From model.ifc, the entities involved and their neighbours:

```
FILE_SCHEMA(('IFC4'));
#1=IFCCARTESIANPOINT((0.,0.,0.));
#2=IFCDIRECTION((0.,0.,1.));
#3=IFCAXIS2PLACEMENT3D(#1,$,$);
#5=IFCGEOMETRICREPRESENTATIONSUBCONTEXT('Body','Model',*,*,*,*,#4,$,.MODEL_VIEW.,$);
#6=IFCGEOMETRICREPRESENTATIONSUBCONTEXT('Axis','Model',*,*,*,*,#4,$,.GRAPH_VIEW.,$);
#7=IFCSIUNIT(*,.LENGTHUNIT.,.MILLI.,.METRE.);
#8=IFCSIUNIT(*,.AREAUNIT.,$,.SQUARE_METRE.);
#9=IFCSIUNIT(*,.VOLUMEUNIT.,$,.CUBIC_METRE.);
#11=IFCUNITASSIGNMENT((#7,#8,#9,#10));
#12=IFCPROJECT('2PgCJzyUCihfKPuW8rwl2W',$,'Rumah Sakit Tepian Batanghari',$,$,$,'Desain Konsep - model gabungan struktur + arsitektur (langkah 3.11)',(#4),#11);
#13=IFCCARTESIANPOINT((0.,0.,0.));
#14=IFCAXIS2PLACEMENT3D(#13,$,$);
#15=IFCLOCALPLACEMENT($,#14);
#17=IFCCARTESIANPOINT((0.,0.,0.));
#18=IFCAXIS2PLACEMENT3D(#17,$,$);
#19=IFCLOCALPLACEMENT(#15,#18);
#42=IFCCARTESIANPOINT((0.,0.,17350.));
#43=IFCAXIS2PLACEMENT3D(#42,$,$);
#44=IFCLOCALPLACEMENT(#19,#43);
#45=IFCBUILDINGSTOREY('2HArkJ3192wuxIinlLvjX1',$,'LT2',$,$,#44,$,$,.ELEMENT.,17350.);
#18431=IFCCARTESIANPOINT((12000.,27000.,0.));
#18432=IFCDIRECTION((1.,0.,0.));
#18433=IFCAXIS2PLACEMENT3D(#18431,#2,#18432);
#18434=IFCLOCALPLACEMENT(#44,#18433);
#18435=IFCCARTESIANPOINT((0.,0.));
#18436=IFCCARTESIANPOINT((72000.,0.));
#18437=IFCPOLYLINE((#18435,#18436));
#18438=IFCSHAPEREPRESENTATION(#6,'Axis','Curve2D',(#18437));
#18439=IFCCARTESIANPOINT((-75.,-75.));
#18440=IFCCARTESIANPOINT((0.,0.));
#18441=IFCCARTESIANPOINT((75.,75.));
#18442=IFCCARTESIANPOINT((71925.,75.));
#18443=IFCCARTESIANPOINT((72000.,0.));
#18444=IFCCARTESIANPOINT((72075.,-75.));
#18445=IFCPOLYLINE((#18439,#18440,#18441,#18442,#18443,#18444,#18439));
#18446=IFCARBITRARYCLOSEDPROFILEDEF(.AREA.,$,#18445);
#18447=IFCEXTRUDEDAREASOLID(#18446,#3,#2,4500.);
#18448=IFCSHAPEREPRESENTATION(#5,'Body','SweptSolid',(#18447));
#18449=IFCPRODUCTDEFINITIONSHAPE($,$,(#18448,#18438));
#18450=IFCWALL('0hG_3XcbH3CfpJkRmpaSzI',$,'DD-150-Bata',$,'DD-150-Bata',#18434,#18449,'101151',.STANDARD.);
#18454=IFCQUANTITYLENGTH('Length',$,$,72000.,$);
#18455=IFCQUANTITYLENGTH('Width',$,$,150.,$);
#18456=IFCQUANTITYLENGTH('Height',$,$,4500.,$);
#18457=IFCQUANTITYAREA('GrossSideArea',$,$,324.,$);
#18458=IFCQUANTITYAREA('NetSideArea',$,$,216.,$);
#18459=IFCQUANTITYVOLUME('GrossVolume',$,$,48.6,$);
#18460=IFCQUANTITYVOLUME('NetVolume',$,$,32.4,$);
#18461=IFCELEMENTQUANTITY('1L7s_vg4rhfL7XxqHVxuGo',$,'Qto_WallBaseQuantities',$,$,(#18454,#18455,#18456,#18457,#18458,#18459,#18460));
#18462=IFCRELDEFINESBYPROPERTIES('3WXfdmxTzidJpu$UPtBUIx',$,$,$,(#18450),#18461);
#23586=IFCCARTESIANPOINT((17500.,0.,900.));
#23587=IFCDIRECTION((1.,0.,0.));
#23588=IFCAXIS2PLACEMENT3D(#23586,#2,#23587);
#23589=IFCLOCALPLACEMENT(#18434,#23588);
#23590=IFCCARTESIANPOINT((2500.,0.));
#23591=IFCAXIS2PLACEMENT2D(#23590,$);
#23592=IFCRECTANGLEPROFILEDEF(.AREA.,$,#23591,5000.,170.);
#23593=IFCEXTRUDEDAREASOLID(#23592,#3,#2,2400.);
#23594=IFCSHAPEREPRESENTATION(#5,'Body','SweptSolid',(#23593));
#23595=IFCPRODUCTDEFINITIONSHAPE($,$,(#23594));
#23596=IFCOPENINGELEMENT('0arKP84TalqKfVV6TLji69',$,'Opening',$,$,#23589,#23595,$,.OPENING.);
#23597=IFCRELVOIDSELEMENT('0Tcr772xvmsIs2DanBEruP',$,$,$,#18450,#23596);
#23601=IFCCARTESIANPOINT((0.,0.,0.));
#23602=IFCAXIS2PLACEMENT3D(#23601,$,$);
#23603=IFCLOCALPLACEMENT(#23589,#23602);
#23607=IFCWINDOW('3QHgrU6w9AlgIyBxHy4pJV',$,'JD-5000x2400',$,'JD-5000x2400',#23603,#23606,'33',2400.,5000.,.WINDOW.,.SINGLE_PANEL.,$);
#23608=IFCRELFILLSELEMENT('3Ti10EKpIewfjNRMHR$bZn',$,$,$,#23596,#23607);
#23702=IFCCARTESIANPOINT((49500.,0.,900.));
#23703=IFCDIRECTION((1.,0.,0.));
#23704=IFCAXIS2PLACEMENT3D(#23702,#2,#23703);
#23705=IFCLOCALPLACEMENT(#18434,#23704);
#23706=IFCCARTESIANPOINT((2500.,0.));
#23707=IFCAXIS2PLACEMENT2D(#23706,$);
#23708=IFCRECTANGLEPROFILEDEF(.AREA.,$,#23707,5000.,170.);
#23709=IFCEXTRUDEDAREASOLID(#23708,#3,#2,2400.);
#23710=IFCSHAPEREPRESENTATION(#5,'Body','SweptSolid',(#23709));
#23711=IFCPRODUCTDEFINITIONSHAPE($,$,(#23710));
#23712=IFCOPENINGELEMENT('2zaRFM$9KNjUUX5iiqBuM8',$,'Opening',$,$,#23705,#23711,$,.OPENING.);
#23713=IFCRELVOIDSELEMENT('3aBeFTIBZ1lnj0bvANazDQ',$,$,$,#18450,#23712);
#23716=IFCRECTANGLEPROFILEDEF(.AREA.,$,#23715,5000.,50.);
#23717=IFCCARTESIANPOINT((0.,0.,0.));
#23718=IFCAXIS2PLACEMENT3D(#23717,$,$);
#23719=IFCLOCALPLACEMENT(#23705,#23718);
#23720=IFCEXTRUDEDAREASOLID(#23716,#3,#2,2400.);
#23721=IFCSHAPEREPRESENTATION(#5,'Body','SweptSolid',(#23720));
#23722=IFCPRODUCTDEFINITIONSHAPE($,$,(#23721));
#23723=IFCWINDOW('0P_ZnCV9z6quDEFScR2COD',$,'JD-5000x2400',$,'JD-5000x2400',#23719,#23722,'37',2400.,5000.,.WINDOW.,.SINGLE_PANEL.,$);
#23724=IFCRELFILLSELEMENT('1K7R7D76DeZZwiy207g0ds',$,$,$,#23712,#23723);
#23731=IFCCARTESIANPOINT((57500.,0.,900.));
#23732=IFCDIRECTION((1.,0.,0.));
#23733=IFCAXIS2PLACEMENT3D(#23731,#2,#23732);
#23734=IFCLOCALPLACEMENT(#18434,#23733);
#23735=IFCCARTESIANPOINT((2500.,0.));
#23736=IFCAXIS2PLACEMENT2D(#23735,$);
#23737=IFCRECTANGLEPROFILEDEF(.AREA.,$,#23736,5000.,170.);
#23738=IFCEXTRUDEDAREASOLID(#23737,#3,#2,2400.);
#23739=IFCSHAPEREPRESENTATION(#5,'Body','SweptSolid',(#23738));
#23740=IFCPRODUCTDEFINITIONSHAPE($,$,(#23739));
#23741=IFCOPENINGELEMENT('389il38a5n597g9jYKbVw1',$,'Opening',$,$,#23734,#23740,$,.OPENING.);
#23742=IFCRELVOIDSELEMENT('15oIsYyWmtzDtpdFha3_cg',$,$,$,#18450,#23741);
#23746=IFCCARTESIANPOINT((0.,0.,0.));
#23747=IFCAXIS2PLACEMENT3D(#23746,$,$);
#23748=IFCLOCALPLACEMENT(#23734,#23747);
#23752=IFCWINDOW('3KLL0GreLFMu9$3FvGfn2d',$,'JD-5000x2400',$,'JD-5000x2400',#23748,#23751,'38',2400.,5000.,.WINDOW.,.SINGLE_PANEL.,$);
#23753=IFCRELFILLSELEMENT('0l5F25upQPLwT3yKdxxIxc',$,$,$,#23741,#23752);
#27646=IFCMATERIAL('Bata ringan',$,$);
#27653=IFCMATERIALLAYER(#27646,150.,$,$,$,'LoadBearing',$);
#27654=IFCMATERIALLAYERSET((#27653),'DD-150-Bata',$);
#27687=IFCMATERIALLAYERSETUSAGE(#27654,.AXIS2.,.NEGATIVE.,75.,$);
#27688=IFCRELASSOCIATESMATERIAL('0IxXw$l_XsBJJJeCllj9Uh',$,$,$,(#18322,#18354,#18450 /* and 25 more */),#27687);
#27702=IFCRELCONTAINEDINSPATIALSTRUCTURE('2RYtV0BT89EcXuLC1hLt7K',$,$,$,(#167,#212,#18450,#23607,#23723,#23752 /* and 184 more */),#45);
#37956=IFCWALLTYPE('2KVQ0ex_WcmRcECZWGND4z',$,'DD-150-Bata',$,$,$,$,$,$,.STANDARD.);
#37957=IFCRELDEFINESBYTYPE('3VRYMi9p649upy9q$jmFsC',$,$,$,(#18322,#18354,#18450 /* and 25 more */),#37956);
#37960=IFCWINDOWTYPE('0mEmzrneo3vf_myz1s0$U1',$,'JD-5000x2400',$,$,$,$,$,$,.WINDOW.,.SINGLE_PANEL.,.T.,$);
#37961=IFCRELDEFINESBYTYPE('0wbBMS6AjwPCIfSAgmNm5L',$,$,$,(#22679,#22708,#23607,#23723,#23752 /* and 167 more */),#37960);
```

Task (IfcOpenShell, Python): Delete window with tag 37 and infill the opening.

```python
import ifcopenshell
import ifcopenshell.api.feature
import ifcopenshell.api.pset
import ifcopenshell.api.root
import ifcopenshell.geom
import ifcopenshell.util.element
import ifcopenshell.util.shape
import ifcopenshell.util.unit

model = ifcopenshell.open("model.ifc")
area_scale = ifcopenshell.util.unit.calculate_unit_scale(model, "AREAUNIT")
volume_scale = ifcopenshell.util.unit.calculate_unit_scale(model, "VOLUMEUNIT")
settings = ifcopenshell.geom.settings()


def volume(element):
    """Net volume in cubic metres, openings subtracted."""
    shape = ifcopenshell.geom.create_shape(settings, element)
    return ifcopenshell.util.shape.get_volume(shape.geometry)


window = model.by_id(23723)
opening = window.FillsVoids[0].RelatingOpeningElement
wall = opening.VoidsElements[0].RelatingBuildingElement
before = volume(wall)

ifcopenshell.api.root.remove_product(model, product=window)
ifcopenshell.api.feature.remove_feature(model, feature=opening)

after = volume(wall)
thickness = 0.15  # wall thickness in metres

# Update the wall's stored quantities.
qto = model.by_id(ifcopenshell.util.element.get_pset(wall, "Qto_WallBaseQuantities", should_inherit=False)["id"])
ifcopenshell.api.pset.edit_qto(model, qto=qto, properties={
    "NetSideArea": after / thickness / area_scale,
    "NetVolume": after / volume_scale,
})

print(f"wall volume {before:.3f} -> {after:.3f} m3")

model.write("model_rev.ifc")
```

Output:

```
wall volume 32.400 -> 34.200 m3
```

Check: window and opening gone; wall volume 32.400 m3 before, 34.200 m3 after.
